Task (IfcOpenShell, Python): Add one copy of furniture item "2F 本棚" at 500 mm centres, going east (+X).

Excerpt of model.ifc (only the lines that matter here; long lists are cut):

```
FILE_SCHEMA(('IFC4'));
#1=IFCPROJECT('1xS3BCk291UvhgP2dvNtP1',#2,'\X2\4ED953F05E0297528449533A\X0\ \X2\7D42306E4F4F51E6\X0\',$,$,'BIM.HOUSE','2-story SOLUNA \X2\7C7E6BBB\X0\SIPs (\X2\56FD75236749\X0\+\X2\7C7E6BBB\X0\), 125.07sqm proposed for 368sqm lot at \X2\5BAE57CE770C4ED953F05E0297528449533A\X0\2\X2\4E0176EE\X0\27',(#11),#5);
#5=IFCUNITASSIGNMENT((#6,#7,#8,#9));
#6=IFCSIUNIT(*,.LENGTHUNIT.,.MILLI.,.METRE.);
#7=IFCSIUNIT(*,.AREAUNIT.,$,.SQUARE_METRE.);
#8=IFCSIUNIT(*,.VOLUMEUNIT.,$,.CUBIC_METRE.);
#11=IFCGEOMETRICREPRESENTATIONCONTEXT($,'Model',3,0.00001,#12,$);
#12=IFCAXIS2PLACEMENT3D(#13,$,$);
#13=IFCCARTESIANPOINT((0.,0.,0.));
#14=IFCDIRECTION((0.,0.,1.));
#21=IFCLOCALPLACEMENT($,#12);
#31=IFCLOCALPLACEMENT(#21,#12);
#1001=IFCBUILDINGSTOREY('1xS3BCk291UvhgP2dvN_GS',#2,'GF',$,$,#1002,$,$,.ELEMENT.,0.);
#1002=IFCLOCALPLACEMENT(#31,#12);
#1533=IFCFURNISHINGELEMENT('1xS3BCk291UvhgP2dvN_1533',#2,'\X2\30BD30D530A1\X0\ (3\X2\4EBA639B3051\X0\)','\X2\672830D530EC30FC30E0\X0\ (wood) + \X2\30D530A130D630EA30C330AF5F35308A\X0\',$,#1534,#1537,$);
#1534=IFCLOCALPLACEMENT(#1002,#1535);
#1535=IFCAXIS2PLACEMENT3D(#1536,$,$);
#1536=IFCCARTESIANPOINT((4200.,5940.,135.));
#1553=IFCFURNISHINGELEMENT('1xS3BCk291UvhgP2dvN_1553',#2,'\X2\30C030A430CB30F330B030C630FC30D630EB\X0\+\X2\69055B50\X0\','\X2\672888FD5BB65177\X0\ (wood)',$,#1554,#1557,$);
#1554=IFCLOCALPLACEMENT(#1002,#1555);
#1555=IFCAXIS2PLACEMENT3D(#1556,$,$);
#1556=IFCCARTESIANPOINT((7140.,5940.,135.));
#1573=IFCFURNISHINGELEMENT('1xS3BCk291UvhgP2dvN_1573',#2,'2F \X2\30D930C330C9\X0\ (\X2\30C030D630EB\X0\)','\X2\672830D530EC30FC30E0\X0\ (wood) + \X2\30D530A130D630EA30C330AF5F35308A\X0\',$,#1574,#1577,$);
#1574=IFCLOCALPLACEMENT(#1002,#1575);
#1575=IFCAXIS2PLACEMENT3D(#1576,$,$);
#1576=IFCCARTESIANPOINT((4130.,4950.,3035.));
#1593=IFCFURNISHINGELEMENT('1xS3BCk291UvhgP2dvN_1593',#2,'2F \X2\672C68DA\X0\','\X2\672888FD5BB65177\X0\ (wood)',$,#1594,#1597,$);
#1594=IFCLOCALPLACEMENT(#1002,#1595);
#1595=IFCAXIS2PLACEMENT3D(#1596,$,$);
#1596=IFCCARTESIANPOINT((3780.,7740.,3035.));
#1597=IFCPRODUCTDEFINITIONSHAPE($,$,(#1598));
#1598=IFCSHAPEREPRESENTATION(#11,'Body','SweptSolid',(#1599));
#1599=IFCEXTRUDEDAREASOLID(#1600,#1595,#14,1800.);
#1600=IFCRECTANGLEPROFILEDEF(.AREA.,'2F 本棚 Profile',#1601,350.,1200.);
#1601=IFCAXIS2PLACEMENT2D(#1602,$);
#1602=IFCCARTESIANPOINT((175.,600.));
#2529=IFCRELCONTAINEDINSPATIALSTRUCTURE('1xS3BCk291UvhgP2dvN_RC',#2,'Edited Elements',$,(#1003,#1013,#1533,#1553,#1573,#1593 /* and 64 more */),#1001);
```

```python
import numpy as np
import ifcopenshell
import ifcopenshell.api.geometry
import ifcopenshell.api.root
import ifcopenshell.util.element
import ifcopenshell.util.placement
import ifcopenshell.util.unit

model = ifcopenshell.open("model.ifc")
unit_scale = ifcopenshell.util.unit.calculate_unit_scale(model)


def reuse_history(source, copy):
    """copy_class also copies each property set's owner history, people and application; keep the originals."""
    for rel in copy.IsDefinedBy:
        if rel.is_a("IfcRelDefinesByProperties") and (history := rel.RelatingPropertyDefinition.OwnerHistory):
            rel.RelatingPropertyDefinition.OwnerHistory = source.OwnerHistory
            ifcopenshell.util.element.remove_deep2(model, history)


source = model.by_guid("1xS3BCk291UvhgP2dvN_1593")
base = ifcopenshell.util.placement.get_local_placement(source.ObjectPlacement)
step = np.array([1.0, 0.0, 0.0]) * 0.5 / unit_scale

for i in range(1, 2):
    copy = ifcopenshell.api.root.copy_class(model, product=source)
    copy.Representation = ifcopenshell.util.element.copy_deep(
        model, source.Representation, exclude=["IfcGeometricRepresentationContext", "IfcRepresentationMap"]
    )
    reuse_history(source, copy)
    matrix = base.copy()
    matrix[:3, 3] += i * step
    print("added at", matrix[:3, 3].round(3) + 0.0)
    ifcopenshell.api.geometry.edit_object_placement(model, product=copy, matrix=matrix, is_si=False)

model.write("model_edited.ifc")
```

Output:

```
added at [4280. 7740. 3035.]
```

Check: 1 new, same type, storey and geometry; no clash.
